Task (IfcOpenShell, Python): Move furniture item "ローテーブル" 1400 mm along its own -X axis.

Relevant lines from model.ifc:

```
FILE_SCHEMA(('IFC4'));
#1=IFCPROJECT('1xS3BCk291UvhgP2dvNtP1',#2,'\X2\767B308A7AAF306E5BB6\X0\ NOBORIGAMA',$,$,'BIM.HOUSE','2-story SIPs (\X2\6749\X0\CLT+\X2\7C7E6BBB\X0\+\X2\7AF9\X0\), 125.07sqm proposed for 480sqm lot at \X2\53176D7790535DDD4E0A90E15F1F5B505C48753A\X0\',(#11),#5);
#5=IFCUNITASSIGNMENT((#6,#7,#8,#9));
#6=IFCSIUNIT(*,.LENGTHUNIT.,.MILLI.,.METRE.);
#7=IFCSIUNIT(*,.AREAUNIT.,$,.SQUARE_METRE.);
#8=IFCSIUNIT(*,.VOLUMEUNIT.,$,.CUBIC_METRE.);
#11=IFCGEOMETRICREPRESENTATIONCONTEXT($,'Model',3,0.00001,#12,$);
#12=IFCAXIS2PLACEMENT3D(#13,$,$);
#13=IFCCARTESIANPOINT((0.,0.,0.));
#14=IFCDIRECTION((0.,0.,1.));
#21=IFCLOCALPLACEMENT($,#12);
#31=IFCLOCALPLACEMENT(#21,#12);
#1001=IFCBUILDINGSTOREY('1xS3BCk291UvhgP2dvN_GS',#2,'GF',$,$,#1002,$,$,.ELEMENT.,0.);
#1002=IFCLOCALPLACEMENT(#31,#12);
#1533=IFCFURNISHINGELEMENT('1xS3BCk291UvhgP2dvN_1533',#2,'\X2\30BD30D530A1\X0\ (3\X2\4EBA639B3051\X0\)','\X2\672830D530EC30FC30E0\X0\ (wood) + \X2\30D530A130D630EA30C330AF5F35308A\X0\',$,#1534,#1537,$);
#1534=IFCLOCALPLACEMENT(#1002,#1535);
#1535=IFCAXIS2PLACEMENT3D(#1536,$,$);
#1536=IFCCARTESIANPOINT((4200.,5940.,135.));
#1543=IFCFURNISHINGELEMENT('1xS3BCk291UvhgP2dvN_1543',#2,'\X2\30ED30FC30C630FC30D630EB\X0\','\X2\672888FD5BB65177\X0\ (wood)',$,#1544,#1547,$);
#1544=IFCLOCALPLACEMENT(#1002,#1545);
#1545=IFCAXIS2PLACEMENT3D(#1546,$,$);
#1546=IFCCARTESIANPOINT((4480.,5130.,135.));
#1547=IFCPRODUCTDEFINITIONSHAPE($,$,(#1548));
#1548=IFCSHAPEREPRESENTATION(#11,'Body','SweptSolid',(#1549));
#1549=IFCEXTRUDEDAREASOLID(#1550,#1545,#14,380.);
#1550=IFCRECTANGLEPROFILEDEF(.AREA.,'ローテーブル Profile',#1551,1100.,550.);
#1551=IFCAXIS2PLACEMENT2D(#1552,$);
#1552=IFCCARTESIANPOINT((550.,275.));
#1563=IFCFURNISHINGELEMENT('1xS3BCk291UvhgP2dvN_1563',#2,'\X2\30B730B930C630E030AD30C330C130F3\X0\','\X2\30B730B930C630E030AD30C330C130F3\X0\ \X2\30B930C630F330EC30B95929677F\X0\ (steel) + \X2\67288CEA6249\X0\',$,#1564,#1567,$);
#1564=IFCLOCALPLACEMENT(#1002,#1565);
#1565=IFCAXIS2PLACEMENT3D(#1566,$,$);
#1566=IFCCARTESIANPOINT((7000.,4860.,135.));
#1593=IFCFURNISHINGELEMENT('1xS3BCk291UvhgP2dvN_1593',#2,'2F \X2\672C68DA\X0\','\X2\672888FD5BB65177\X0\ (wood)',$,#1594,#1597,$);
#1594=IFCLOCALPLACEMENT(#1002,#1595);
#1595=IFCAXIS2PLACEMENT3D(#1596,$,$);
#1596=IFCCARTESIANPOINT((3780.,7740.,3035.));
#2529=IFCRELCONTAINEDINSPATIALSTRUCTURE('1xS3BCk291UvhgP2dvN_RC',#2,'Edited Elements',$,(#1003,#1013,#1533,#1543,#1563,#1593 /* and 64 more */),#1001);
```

```python
import ifcopenshell
import ifcopenshell.api.geometry
import ifcopenshell.util.placement

model = ifcopenshell.open("model.ifc")

item = model.by_guid("1xS3BCk291UvhgP2dvN_1543")
matrix = ifcopenshell.util.placement.get_local_placement(item.ObjectPlacement)
matrix[:3, 3] -= matrix[:3, 0] * 1400.0
ifcopenshell.api.geometry.edit_object_placement(model, product=item, matrix=matrix, is_si=False)

print(ifcopenshell.util.placement.get_local_placement(item.ObjectPlacement).round(3) + 0.0)

model.write("model_updated.ifc")
```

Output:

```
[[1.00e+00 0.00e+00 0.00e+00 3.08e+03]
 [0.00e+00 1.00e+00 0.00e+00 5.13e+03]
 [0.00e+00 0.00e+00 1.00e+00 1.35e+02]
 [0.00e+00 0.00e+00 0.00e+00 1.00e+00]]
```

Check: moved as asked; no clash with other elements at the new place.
